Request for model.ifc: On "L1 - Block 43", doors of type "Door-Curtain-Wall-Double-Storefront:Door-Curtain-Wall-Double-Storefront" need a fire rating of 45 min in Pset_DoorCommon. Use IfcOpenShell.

First a look at what the model holds.

```python
import ifcopenshell
import ifcopenshell.util.element

model = ifcopenshell.open("model.ifc")
print(model.schema)
storey = next(s for s in model.by_type("IfcBuildingStorey") if s.Name == "L1 - Block 43")
doors = [e for e in ifcopenshell.util.element.get_decomposition(storey) if e.is_a("IfcDoor")]
seen = {}
for e in doors:
    element_type = ifcopenshell.util.element.get_type(e)
    key = (element_type.Name if element_type != e and element_type else None, ifcopenshell.util.element.get_pset(e, "Pset_DoorCommon", "FireRating"))
    seen[key] = seen.get(key, 0) + 1
for (name, value), count in sorted(seen.items(), key=str):
    print(count, "x", name, "|", value)
```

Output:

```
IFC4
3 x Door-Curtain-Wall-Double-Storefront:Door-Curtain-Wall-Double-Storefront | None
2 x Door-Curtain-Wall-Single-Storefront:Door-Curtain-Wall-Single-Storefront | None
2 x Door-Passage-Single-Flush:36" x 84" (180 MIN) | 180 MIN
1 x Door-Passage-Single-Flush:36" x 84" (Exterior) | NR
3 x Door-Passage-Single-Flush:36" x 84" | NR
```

```python
import ifcopenshell
import ifcopenshell.api.pset
import ifcopenshell.util.element

model = ifcopenshell.open("model.ifc")

storey = next(s for s in model.by_type("IfcBuildingStorey") if s.Name == "L1 - Block 43")
doors = [e for e in ifcopenshell.util.element.get_decomposition(storey) if e.is_a("IfcDoor")]

count = 0
for e in doors:
    element_type = ifcopenshell.util.element.get_type(e)
    if element_type in (None, e) or element_type.Name != "Door-Curtain-Wall-Double-Storefront:Door-Curtain-Wall-Double-Storefront":
        continue
    # add_pset returns the element's existing set when there is one.
    pset = ifcopenshell.api.pset.add_pset(model, product=e, name="Pset_DoorCommon")
    ifcopenshell.api.pset.edit_pset(model, pset=pset, properties={"FireRating": "45 min"})
    count += 1

print(count, "doors updated")

model.write("model-out.ifc")
```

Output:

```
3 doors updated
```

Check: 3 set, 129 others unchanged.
